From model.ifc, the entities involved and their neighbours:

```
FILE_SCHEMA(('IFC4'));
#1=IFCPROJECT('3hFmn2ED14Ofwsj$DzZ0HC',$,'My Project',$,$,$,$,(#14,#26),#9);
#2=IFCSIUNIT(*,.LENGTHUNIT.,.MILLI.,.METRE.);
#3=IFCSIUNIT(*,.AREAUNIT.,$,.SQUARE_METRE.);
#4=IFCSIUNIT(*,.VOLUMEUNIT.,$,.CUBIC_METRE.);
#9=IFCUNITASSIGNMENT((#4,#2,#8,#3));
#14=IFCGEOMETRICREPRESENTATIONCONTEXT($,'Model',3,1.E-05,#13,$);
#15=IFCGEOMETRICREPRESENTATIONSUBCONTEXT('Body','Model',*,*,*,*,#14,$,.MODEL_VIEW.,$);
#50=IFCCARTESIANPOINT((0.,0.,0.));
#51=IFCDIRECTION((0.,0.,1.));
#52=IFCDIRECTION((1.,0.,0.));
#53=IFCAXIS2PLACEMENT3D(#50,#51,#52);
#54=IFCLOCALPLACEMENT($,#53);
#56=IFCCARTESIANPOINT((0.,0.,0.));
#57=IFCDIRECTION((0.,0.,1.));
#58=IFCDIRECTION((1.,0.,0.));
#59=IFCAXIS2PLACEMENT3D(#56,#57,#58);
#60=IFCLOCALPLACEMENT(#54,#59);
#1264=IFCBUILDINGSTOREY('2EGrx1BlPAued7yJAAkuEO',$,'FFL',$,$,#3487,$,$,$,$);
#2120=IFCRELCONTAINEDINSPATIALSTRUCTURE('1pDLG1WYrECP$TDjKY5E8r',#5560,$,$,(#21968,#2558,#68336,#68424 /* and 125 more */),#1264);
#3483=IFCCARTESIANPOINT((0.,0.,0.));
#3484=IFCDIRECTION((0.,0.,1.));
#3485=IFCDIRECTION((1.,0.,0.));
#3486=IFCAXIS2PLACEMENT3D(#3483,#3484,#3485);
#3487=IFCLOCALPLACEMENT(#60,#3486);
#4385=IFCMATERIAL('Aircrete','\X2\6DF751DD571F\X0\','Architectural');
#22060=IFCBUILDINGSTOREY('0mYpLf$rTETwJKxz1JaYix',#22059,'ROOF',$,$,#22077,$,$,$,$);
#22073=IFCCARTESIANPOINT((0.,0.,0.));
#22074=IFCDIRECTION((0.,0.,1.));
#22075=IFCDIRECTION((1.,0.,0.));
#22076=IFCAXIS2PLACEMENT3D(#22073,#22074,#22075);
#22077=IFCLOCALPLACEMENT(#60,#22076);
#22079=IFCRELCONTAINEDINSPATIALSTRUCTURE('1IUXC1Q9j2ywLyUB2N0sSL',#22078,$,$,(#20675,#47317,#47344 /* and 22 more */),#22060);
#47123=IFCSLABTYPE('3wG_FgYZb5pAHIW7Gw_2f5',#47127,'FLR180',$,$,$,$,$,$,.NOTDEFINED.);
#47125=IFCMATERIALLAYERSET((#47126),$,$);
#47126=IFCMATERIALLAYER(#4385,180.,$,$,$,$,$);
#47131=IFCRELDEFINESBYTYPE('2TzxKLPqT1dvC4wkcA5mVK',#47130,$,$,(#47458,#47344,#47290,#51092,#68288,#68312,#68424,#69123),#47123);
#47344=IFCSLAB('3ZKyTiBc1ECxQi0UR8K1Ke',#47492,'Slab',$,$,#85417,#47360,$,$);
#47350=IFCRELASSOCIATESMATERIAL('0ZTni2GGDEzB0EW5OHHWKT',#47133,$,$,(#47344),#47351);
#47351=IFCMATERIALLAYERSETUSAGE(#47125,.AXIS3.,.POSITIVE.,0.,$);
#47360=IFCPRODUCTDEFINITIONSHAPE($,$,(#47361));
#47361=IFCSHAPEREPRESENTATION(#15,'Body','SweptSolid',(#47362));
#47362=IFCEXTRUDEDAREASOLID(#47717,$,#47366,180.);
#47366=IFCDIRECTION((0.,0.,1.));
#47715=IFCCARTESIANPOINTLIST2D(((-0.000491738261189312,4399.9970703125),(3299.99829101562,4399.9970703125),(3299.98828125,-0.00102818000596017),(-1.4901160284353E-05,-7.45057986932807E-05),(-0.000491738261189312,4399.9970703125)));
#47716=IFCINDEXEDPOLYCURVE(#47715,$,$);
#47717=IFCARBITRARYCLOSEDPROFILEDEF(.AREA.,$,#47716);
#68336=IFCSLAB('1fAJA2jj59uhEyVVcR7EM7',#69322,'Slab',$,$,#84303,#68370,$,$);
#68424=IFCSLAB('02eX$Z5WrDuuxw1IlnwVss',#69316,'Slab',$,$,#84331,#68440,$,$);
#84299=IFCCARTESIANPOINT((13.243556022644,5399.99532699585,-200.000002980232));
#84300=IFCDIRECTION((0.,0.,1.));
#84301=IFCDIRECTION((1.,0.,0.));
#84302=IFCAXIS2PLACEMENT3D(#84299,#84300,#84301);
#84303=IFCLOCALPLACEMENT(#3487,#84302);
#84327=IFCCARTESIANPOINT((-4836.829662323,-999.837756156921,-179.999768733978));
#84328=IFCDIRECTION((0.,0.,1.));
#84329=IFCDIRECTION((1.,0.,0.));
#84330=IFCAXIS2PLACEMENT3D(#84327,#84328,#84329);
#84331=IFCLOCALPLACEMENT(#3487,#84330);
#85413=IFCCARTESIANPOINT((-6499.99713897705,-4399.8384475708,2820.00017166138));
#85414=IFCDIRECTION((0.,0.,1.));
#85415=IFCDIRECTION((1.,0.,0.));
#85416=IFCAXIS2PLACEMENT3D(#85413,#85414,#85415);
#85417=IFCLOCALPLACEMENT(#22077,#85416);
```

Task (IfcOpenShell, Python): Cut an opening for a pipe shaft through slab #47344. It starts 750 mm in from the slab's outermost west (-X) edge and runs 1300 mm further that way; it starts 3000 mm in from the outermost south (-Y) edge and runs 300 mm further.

```python
import numpy as np
import ifcopenshell
import ifcopenshell.api.feature
import ifcopenshell.api.geometry
import ifcopenshell.api.root
import ifcopenshell.geom
import ifcopenshell.util.placement
import ifcopenshell.util.representation
import ifcopenshell.util.shape
import ifcopenshell.util.unit

model = ifcopenshell.open("model.ifc")
unit_scale = ifcopenshell.util.unit.calculate_unit_scale(model)
settings = ifcopenshell.geom.settings()


def volume(element):
    """Net volume in cubic metres, openings subtracted."""
    shape = ifcopenshell.geom.create_shape(settings, element)
    return ifcopenshell.util.shape.get_volume(shape.geometry)


slab = model.by_id(47344)
before = volume(slab)

# Extent in the slab's own axes, in metres. The edges named are its -X and -Y sides.
slab_shape = ifcopenshell.geom.create_shape(settings, slab)
vertices = ifcopenshell.util.shape.get_vertices(slab_shape.geometry)
x_min, y_min, bottom = vertices.min(axis=0)
top = vertices[:, 2].max()

opening = ifcopenshell.api.root.create_entity(model, ifc_class="IfcOpeningElement", name="Pipe shaft opening", predefined_type="OPENING")
context = ifcopenshell.util.representation.get_context(model, "Model", "Body", "MODEL_VIEW")
width, depth = 1.3, 0.3
outline = [(0.0, 0.0), (width, 0.0), (width, depth), (0.0, depth), (0.0, 0.0)]
# Overshoot both faces by 50 mm so the cut is clean.
shape = ifcopenshell.api.geometry.add_slab_representation(
    model, context=context, depth=top - bottom + 0.1, polyline=outline
)
ifcopenshell.api.geometry.assign_representation(model, product=opening, representation=shape)

matrix = ifcopenshell.util.placement.get_local_placement(slab.ObjectPlacement)
matrix[:, 3] = matrix @ np.append(np.array([x_min + 0.75, y_min + 3, bottom - 0.05]) / unit_scale, 1.0)
ifcopenshell.api.geometry.edit_object_placement(model, product=opening, matrix=matrix, is_si=False)
ifcopenshell.api.feature.add_feature(model, feature=opening, element=slab)

after = volume(slab)

print(f"slab volume {before:.3f} -> {after:.3f} m3")

model.write("model_updated.ifc")
```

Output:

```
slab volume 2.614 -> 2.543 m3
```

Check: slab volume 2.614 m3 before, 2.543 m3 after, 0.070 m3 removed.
